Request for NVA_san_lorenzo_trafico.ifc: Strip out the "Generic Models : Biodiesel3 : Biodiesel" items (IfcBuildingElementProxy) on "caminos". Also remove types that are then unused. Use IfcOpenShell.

First a look at what the model holds.

```python
import ifcopenshell
import ifcopenshell.util.element

model = ifcopenshell.open("NVA_san_lorenzo_trafico.ifc")
print(model.schema)
storey = next(s for s in model.by_type("IfcBuildingStorey") if s.Name == "caminos")
proxies = [e for e in ifcopenshell.util.element.get_decomposition(storey) if e.is_a("IfcBuildingElementProxy")]
seen = {}
for e in proxies:
    element_type = ifcopenshell.util.element.get_type(e)
    name = element_type.Name if element_type not in (None, e) else None
    seen[name] = seen.get(name, 0) + 1
for name, count in sorted(seen.items(), key=str):
    print(count, "x", name)
```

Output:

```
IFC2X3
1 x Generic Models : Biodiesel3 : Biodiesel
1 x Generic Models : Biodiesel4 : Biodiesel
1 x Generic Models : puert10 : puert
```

```python
import ifcopenshell
import ifcopenshell.api.root
import ifcopenshell.util.element

model = ifcopenshell.open("NVA_san_lorenzo_trafico.ifc")

storey = next(s for s in model.by_type("IfcBuildingStorey") if s.Name == "caminos")
proxies = [e for e in ifcopenshell.util.element.get_decomposition(storey) if e.is_a("IfcBuildingElementProxy")]
targets = [e for e in proxies if (t := ifcopenshell.util.element.get_type(e)) not in (None, e) and t.Name == "Generic Models : Biodiesel3 : Biodiesel"]
types = {ifcopenshell.util.element.get_type(e) for e in targets} - {None, *targets}

for e in targets:
    ifcopenshell.api.root.remove_product(model, product=e)
print(len(targets), "removed")

unused = [t for t in types if not ifcopenshell.util.element.get_types(t)]
for t in unused:
    ifcopenshell.api.root.remove_product(model, product=t)
print(len(unused), "unused types removed")

model.write("NVA_san_lorenzo_trafico_rev.ifc")
```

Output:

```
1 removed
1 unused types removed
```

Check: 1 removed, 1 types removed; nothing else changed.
